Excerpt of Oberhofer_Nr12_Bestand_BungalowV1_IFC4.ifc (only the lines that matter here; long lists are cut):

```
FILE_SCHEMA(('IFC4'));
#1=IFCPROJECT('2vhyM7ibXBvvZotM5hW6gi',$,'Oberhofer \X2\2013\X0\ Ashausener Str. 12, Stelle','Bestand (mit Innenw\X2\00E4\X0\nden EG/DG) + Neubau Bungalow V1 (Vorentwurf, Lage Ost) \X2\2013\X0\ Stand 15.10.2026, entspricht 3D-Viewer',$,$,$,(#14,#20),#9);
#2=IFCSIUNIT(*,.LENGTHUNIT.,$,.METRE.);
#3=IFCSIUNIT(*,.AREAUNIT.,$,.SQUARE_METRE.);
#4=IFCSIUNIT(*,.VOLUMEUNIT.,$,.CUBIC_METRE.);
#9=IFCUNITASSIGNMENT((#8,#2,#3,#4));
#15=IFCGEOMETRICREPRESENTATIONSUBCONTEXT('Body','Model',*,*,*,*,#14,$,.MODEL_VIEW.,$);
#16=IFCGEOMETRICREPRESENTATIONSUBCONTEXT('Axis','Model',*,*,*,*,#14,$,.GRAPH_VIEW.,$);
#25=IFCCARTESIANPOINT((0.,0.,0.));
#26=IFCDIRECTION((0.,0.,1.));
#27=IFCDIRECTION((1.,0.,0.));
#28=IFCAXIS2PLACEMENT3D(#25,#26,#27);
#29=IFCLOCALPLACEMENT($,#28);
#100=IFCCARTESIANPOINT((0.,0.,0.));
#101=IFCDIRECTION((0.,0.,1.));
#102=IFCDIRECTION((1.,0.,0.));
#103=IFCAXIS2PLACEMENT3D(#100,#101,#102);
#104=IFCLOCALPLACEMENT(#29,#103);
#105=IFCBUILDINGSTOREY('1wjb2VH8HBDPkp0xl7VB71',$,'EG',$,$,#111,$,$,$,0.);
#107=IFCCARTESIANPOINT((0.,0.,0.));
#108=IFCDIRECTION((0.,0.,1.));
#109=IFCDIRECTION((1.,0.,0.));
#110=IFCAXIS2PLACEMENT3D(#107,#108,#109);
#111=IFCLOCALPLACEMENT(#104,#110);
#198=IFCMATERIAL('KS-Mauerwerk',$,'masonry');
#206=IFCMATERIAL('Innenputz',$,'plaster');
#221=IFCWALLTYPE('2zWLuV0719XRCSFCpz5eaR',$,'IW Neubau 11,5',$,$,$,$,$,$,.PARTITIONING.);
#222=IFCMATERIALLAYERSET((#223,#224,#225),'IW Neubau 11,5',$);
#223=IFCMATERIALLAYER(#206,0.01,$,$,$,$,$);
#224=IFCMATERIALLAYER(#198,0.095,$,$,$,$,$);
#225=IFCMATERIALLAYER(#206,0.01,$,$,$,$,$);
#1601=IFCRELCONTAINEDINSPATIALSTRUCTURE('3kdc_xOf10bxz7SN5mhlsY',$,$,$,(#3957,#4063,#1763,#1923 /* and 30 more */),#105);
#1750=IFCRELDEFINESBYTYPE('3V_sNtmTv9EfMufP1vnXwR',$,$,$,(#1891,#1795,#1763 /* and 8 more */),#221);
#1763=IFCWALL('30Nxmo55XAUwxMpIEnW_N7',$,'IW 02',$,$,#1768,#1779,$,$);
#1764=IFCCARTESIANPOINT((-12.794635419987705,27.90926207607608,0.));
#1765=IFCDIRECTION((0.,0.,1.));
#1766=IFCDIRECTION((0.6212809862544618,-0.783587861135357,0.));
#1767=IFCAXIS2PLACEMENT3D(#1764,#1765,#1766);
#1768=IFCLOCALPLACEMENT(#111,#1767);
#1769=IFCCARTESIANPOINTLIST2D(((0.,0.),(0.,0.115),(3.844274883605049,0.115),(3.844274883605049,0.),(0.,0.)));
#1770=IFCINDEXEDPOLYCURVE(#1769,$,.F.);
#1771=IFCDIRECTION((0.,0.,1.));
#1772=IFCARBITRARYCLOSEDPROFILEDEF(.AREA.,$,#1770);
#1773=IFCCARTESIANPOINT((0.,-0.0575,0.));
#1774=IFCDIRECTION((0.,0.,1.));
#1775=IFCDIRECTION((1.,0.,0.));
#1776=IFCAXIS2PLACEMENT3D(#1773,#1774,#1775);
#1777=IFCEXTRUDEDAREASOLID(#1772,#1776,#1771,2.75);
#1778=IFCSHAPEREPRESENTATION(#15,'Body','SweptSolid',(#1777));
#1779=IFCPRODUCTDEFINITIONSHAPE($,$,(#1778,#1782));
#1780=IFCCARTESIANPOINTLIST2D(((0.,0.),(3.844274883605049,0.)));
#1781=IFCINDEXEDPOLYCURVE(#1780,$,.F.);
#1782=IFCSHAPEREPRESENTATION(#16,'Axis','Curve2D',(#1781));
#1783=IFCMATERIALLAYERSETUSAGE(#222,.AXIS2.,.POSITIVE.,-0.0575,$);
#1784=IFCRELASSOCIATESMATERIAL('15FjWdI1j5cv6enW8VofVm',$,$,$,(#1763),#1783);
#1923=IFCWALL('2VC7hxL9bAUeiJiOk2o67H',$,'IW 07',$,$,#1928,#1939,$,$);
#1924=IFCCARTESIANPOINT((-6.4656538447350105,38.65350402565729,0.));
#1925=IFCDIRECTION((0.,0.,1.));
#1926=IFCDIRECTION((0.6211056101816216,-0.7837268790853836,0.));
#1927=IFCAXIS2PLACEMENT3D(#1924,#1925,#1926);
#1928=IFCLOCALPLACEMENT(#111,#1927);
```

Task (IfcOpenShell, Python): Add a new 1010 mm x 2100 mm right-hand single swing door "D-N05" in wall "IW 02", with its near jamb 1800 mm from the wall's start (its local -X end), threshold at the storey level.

```python
import numpy as np
import ifcopenshell
import ifcopenshell.api.feature
import ifcopenshell.api.geometry
import ifcopenshell.api.root
import ifcopenshell.api.spatial
import ifcopenshell.geom
import ifcopenshell.util.element
import ifcopenshell.util.placement
import ifcopenshell.util.representation
import ifcopenshell.util.shape
import ifcopenshell.util.unit

model = ifcopenshell.open("Oberhofer_Nr12_Bestand_BungalowV1_IFC4.ifc")
unit_scale = ifcopenshell.util.unit.calculate_unit_scale(model)
settings = ifcopenshell.geom.settings()


def volume(element):
    """Net volume in cubic metres, openings subtracted."""
    shape = ifcopenshell.geom.create_shape(settings, element)
    return ifcopenshell.util.shape.get_volume(shape.geometry)


wall = model.by_guid("30Nxmo55XAUwxMpIEnW_N7")
storey = ifcopenshell.util.element.get_container(wall, ifc_class="IfcBuildingStorey")
context = ifcopenshell.util.representation.get_context(model, "Model", "Body", "MODEL_VIEW")
before = volume(wall)

width, height, from_end, sill = 1.01, 2.1, 1.8, 0.0  # metres

# The wall runs along its own X axis, and the end named is its -X end.
wall_shape = ifcopenshell.geom.create_shape(settings, wall)
x, y, z = ifcopenshell.util.shape.get_vertices(wall_shape.geometry).T
start = x.min() + from_end
face, thickness = float(y.min()), float(y.max() - y.min())
wall_matrix = ifcopenshell.util.placement.get_local_placement(wall.ObjectPlacement)
level = ifcopenshell.util.placement.get_local_placement(storey.ObjectPlacement)[2, 3]


def in_wall(x, y):
    """Placement at x, y metres in the wall's axes, at sill height."""
    matrix = wall_matrix.copy()
    matrix[:, 3] = wall_matrix @ np.array([x / unit_scale, y / unit_scale, 0.0, 1.0])
    matrix[2, 3] = level + sill / unit_scale
    return matrix


# Opening: a box that overshoots both wall faces by 50 mm.
opening = ifcopenshell.api.root.create_entity(model, ifc_class="IfcOpeningElement", predefined_type="OPENING")
box = ifcopenshell.api.geometry.add_wall_representation(
    model, context=context, length=width, height=height, thickness=thickness + 0.1
)
ifcopenshell.api.geometry.assign_representation(model, product=opening, representation=box)
ifcopenshell.api.geometry.edit_object_placement(model, product=opening, matrix=in_wall(start, face - 0.05), is_si=False)
ifcopenshell.api.feature.add_feature(model, feature=opening, element=wall)

door = ifcopenshell.api.root.create_entity(model, ifc_class="IfcDoor", name="D-N05", predefined_type="DOOR")
door.OverallWidth, door.OverallHeight = width / unit_scale, height / unit_scale
door.OperationType = "SINGLE_SWING_RIGHT"
body = ifcopenshell.api.geometry.add_door_representation(
    model,
    context=context,
    overall_width=door.OverallWidth,
    overall_height=door.OverallHeight,
    operation_type="SINGLE_SWING_RIGHT",
    lining_properties={"LiningDepth": thickness / unit_scale, "ThresholdDepth": thickness / unit_scale},
)
ifcopenshell.api.geometry.assign_representation(model, product=door, representation=body)
ifcopenshell.api.spatial.assign_container(model, products=[door], relating_structure=storey)
ifcopenshell.api.feature.add_filling(model, opening=opening, element=door)

# The lining spans the wall, so the door starts at the wall face.
ifcopenshell.api.geometry.edit_object_placement(model, product=door, matrix=in_wall(start, face), is_si=False)

after = volume(wall)

print(f"wall volume {before:.3f} -> {after:.3f} m3")

model.write("Oberhofer_Nr12_Bestand_BungalowV1_IFC4_v2.ifc")
```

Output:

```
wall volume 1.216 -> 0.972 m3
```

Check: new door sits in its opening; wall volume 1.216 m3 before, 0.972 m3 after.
